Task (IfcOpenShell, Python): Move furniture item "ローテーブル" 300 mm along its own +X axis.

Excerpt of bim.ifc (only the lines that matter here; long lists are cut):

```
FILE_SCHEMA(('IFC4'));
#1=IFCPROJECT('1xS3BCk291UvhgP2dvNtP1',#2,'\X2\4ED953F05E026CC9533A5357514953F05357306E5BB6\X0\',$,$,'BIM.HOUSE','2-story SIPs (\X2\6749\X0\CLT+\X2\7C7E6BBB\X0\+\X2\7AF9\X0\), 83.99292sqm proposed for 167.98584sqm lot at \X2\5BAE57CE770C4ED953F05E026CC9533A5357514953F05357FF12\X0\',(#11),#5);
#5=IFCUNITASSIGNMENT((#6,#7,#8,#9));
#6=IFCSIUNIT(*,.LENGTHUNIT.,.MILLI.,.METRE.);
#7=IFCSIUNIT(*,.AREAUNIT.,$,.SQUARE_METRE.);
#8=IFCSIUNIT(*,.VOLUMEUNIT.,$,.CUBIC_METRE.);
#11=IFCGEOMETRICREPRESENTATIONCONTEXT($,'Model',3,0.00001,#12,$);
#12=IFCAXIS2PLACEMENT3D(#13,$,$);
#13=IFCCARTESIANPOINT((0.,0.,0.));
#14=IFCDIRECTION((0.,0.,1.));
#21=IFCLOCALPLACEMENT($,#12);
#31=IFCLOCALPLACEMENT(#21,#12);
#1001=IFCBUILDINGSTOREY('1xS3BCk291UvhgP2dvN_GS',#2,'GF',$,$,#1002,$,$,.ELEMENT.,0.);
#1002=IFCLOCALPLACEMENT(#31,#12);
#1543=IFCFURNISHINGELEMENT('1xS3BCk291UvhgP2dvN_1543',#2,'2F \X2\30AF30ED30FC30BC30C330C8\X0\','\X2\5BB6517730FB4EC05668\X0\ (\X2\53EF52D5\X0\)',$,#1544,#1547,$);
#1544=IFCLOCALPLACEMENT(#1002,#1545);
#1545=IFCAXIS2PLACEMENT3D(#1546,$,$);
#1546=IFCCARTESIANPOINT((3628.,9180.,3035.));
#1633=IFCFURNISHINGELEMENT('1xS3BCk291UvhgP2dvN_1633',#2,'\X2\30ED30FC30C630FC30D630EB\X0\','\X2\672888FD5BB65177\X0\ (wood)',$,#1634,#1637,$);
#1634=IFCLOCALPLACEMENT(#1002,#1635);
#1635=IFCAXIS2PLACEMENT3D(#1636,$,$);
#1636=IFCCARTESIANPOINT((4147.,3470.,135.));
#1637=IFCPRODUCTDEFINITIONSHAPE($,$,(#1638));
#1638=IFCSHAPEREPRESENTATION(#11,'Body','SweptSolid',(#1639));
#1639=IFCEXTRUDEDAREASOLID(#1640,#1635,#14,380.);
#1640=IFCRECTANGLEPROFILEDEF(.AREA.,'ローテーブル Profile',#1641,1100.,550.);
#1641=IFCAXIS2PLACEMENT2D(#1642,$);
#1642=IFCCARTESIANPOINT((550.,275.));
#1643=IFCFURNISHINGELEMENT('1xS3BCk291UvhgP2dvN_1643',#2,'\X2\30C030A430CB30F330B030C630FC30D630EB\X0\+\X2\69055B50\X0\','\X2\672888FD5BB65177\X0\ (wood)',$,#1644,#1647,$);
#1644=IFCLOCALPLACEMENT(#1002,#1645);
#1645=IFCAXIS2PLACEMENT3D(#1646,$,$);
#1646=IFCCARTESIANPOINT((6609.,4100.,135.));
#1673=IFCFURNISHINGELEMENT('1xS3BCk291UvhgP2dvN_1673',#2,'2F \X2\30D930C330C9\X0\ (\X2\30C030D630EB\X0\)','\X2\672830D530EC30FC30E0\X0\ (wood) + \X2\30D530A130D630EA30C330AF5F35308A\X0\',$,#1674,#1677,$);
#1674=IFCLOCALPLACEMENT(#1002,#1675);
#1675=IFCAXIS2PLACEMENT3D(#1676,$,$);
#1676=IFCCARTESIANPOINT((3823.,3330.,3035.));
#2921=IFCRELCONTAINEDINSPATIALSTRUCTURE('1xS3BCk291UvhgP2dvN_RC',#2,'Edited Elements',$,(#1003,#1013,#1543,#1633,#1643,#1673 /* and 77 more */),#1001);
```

```python
import ifcopenshell
import ifcopenshell.api.geometry
import ifcopenshell.util.placement
import ifcopenshell.util.unit

model = ifcopenshell.open("bim.ifc")
unit_scale = ifcopenshell.util.unit.calculate_unit_scale(model)

item = model.by_guid("1xS3BCk291UvhgP2dvN_1633")
matrix = ifcopenshell.util.placement.get_local_placement(item.ObjectPlacement)
matrix[:3, 3] += matrix[:3, 0] * 0.3 / unit_scale
ifcopenshell.api.geometry.edit_object_placement(model, product=item, matrix=matrix, is_si=False)

print(ifcopenshell.util.placement.get_local_placement(item.ObjectPlacement).round(3) + 0.0)

model.write("bim_rev.ifc")
```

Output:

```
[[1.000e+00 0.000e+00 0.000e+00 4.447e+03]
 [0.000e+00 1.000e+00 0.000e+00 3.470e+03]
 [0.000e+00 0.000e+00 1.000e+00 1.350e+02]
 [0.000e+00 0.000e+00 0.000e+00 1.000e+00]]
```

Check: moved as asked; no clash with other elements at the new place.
